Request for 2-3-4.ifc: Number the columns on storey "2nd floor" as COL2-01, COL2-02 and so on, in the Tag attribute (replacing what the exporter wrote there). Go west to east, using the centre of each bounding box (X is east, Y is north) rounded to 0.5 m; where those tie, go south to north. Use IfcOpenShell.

First a look at what the model holds.

```python
import ifcopenshell
import ifcopenshell.util.element
import ifcopenshell.util.placement

model = ifcopenshell.open("2-3-4.ifc")
print(model.schema)
storey = next(s for s in model.by_type("IfcBuildingStorey") if s.Name == "2nd floor")
columns = [e for e in ifcopenshell.util.element.get_decomposition(storey) if e.is_a("IfcColumn")]
for e in sorted(columns, key=lambda e: e.id()):
    origin = ifcopenshell.util.placement.get_local_placement(e.ObjectPlacement)[:3, 3]
    print(e.id(), e.Tag, e.Name, origin.round(2) + 0.0, sep=" | ")
```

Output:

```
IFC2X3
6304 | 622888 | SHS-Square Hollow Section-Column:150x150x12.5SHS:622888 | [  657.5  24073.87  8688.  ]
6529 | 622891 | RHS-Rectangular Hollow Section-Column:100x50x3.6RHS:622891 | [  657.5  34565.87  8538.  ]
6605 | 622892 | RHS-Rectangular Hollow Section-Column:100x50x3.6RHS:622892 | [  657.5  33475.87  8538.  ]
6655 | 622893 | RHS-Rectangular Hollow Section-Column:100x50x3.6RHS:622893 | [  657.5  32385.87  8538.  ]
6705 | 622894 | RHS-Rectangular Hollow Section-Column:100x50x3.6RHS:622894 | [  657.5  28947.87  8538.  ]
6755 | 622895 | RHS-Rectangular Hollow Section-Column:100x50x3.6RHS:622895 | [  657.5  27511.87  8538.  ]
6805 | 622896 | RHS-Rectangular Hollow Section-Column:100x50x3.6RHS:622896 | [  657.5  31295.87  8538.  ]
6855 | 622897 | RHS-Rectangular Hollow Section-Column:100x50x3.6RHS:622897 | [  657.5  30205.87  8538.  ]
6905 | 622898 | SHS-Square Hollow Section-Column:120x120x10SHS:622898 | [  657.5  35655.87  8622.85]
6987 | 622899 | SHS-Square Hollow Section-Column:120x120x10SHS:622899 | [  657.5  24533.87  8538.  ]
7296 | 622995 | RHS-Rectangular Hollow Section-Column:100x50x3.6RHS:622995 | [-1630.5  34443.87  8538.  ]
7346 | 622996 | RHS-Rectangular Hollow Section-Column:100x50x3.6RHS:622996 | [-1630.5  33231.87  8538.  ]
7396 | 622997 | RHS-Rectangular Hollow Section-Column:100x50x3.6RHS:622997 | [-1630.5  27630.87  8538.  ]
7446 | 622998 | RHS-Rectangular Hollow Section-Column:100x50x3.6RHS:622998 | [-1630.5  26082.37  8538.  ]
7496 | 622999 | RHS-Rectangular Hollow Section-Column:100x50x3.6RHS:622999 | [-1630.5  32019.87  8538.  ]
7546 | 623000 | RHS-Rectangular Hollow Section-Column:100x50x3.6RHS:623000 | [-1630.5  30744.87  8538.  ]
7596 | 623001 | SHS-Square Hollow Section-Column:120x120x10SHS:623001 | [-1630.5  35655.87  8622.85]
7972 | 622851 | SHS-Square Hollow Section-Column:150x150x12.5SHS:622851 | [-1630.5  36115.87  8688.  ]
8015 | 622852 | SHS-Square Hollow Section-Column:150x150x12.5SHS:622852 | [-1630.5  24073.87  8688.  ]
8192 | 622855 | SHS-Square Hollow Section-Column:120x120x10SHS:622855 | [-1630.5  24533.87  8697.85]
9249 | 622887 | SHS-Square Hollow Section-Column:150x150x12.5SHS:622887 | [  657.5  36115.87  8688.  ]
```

```python
import ifcopenshell
import ifcopenshell.geom
import ifcopenshell.util.element
import ifcopenshell.util.shape

model = ifcopenshell.open("2-3-4.ifc")
settings = ifcopenshell.geom.settings()
settings.set("use-world-coords", True)


def centre(element):
    shape = ifcopenshell.geom.create_shape(settings, element)
    return ifcopenshell.util.shape.get_bbox_centroid(shape.geometry)


storey = next(s for s in model.by_type("IfcBuildingStorey") if s.Name == "2nd floor")
columns = [e for e in ifcopenshell.util.element.get_decomposition(storey) if e.is_a("IfcColumn")]

# Insertion points can sit at a corner or the storey origin, so sort by the geometry (in metres).
centres = {e: centre(e) for e in columns}
columns.sort(key=lambda e: (round(centres[e][0] / 0.5), centres[e][1]))

for i, e in enumerate(columns, start=1):
    number = f"COL2-{i:02d}"
    e.Tag = number
    print(e.id(), number)

model.write("2-3-4_rev.ifc")
```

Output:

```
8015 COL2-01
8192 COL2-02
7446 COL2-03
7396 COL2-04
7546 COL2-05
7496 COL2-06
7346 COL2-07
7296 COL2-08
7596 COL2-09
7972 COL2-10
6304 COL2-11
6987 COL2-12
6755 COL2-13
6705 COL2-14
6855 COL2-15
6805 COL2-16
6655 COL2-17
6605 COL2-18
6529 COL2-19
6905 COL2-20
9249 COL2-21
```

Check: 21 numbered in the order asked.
